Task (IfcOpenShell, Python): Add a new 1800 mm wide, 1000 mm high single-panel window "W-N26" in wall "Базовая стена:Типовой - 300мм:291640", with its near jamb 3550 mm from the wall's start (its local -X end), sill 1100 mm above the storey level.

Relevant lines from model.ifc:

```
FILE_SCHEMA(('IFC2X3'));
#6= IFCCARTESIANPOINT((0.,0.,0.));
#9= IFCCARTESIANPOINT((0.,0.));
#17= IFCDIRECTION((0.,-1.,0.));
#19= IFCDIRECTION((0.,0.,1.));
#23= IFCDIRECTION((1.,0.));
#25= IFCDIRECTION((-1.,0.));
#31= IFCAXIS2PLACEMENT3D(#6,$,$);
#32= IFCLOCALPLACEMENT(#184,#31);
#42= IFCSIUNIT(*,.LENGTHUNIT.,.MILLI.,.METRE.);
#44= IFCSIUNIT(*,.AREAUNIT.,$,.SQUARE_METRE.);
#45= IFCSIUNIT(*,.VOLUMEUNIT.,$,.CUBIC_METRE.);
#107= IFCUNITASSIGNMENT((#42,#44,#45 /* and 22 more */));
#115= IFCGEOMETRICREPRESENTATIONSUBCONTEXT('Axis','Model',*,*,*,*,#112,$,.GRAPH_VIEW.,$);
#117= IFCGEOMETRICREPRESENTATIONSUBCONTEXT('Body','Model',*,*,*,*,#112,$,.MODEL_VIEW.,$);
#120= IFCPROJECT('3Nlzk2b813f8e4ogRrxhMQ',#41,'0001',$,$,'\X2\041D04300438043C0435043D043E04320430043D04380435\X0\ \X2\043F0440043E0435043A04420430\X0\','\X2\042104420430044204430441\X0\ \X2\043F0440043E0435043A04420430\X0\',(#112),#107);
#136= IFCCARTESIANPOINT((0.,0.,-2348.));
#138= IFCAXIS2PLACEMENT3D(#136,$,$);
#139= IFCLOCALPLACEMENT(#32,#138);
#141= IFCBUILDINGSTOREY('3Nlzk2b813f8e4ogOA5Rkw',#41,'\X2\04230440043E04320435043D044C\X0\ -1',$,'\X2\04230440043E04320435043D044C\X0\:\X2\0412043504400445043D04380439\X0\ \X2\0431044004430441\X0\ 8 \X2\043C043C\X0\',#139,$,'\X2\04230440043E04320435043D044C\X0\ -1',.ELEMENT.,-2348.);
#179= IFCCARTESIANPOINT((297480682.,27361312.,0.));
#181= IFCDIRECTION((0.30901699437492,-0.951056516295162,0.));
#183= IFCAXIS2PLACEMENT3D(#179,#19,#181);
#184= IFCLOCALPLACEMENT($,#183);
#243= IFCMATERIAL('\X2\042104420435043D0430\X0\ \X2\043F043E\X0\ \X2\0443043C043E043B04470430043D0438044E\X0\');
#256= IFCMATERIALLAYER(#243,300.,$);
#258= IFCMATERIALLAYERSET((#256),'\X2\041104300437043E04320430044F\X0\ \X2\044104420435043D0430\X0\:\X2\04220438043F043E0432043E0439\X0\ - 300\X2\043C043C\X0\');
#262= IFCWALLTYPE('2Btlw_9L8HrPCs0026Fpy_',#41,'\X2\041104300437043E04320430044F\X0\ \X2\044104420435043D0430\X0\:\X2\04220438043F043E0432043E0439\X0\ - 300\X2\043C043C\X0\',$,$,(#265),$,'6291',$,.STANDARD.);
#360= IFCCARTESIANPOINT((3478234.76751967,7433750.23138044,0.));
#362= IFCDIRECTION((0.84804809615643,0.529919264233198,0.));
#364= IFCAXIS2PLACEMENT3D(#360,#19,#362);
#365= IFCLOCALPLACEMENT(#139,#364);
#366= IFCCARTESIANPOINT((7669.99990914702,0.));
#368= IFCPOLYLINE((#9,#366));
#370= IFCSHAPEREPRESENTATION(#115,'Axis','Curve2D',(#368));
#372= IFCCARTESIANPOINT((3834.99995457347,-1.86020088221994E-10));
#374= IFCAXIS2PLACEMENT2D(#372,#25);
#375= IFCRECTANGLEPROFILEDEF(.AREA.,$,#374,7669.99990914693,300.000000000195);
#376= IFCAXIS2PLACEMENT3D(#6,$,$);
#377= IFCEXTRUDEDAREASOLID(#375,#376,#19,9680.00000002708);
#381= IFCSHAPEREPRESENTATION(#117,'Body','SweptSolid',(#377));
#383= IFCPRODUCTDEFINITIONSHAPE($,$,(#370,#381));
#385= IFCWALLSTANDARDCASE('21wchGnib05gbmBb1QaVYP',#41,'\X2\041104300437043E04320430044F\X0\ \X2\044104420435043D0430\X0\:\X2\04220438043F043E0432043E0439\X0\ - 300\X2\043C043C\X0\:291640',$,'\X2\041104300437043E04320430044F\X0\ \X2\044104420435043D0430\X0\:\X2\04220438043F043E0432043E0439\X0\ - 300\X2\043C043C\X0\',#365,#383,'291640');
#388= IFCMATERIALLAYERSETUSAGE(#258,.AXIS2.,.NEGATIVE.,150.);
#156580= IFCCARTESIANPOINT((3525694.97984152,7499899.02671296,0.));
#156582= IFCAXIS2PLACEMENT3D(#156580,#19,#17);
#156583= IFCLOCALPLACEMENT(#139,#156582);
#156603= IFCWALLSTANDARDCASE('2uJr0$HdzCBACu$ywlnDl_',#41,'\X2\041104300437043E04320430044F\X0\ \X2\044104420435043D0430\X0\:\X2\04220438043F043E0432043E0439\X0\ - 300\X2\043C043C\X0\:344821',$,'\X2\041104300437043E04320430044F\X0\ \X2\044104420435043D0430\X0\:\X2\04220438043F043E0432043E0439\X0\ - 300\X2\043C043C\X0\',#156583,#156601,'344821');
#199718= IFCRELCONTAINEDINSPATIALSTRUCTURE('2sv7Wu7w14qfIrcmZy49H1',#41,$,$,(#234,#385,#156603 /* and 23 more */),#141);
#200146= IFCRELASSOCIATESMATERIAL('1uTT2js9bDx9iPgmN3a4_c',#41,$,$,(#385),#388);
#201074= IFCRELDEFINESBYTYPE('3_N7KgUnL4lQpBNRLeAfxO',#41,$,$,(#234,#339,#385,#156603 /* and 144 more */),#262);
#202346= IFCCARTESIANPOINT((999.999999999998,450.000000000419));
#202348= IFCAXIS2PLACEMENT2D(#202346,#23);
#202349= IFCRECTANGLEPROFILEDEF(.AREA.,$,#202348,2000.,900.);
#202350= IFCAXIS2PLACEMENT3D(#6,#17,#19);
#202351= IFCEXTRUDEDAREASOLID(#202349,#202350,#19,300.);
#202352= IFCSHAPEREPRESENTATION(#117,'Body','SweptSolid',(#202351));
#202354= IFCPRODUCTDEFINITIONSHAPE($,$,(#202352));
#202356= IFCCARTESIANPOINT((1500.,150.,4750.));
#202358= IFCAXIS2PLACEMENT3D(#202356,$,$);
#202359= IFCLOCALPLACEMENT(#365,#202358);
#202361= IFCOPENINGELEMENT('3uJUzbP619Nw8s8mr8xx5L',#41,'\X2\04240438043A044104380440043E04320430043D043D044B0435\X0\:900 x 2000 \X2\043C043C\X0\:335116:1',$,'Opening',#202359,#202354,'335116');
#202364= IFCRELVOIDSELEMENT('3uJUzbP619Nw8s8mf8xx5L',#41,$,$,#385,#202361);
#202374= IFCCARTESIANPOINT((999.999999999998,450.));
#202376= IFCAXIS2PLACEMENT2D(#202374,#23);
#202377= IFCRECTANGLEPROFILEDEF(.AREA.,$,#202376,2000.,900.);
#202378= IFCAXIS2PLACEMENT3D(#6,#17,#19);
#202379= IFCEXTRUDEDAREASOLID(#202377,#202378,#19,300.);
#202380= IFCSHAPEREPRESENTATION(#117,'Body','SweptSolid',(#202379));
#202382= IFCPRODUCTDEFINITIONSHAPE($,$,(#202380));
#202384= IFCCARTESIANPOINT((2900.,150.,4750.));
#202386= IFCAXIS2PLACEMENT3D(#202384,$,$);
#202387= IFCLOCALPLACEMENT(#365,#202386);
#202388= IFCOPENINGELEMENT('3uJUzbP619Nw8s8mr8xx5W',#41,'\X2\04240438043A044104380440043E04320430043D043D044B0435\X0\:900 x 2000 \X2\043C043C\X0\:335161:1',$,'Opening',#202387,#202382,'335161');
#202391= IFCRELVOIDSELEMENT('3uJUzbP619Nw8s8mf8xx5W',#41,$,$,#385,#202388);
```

```python
import numpy as np
import ifcopenshell
import ifcopenshell.api.feature
import ifcopenshell.api.geometry
import ifcopenshell.api.root
import ifcopenshell.api.spatial
import ifcopenshell.api.type
import ifcopenshell.geom
import ifcopenshell.util.element
import ifcopenshell.util.placement
import ifcopenshell.util.representation
import ifcopenshell.util.shape
import ifcopenshell.util.unit

model = ifcopenshell.open("model.ifc")
unit_scale = ifcopenshell.util.unit.calculate_unit_scale(model)
settings = ifcopenshell.geom.settings()


def volume(element):
    """Net volume in cubic metres, openings subtracted."""
    shape = ifcopenshell.geom.create_shape(settings, element)
    return ifcopenshell.util.shape.get_volume(shape.geometry)


wall = model.by_guid("21wchGnib05gbmBb1QaVYP")
storey = ifcopenshell.util.element.get_container(wall, ifc_class="IfcBuildingStorey")
context = ifcopenshell.util.representation.get_context(model, "Model", "Body", "MODEL_VIEW")
before = volume(wall)

width, height, from_end, sill = 1.8, 1, 3.55, 1.1  # metres

# The wall runs along its own X axis, and the end named is its -X end.
wall_shape = ifcopenshell.geom.create_shape(settings, wall)
x, y, z = ifcopenshell.util.shape.get_vertices(wall_shape.geometry).T
start = x.min() + from_end
face, thickness = float(y.min()), float(y.max() - y.min())
wall_matrix = ifcopenshell.util.placement.get_local_placement(wall.ObjectPlacement)
level = ifcopenshell.util.placement.get_local_placement(storey.ObjectPlacement)[2, 3]


def in_wall(x, y):
    """Placement at x, y metres in the wall's axes, at sill height."""
    matrix = wall_matrix.copy()
    matrix[:, 3] = wall_matrix @ np.array([x / unit_scale, y / unit_scale, 0.0, 1.0])
    matrix[2, 3] = level + sill / unit_scale
    return matrix


# Opening: a box that overshoots both wall faces by 50 mm.
opening = ifcopenshell.api.root.create_entity(model, ifc_class="IfcOpeningElement")
box = ifcopenshell.api.geometry.add_wall_representation(
    model, context=context, length=width, height=height, thickness=thickness + 0.1
)
ifcopenshell.api.geometry.assign_representation(model, product=opening, representation=box)
ifcopenshell.api.geometry.edit_object_placement(model, product=opening, matrix=in_wall(start, face - 0.05), is_si=False)
ifcopenshell.api.feature.add_feature(model, feature=opening, element=wall)

window = ifcopenshell.api.root.create_entity(model, ifc_class="IfcWindow", name="W-N26")
window.OverallWidth, window.OverallHeight = width / unit_scale, height / unit_scale
body = ifcopenshell.api.geometry.add_window_representation(
    model,
    context=context,
    overall_width=window.OverallWidth,
    overall_height=window.OverallHeight,
    partition_type="SINGLE_PANEL",
)
ifcopenshell.api.geometry.assign_representation(model, product=window, representation=body)
ifcopenshell.api.spatial.assign_container(model, products=[window], relating_structure=storey)
fills = ifcopenshell.api.feature.add_filling(model, opening=opening, element=window)
fills.OwnerHistory = window.OwnerHistory  # required in IFC2X3

# IFC2X3 keeps the operation on the window style.
style = ifcopenshell.api.root.create_entity(model, ifc_class="IfcWindowStyle", name="W-N26")
style.OperationType, style.ConstructionType = "SINGLE_PANEL", "NOTDEFINED"
style.ParameterTakesPrecedence = style.Sizeable = False
ifcopenshell.api.type.assign_type(model, related_objects=[window], relating_type=style)

# Centre the window in the wall's thickness.
ifcopenshell.api.geometry.edit_object_placement(model, product=window, matrix=in_wall(start, face), is_si=False)
window_shape = ifcopenshell.geom.create_shape(settings, window)
depth = ifcopenshell.util.shape.get_vertices(window_shape.geometry)[:, 1]
offset = face + thickness / 2 - (depth.min() + depth.max()) / 2
ifcopenshell.api.geometry.edit_object_placement(model, product=window, matrix=in_wall(start, offset), is_si=False)

after = volume(wall)

print(f"wall volume {before:.3f} -> {after:.3f} m3")

model.write("model_updated.ifc")
```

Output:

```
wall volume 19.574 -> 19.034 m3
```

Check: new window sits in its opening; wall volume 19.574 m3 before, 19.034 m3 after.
